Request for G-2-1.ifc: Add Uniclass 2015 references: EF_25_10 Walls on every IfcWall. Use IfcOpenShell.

First a look at what the model holds.

```python
import ifcopenshell

model = ifcopenshell.open("G-2-1.ifc")
print(model.schema)
print("classifications:", [c.Name for c in model.by_type("IfcClassification")])
for ifc_class in ("IfcDoor", "IfcRoof", "IfcStair", "IfcWall", "IfcWindow"):
    print(ifc_class, len(model.by_type(ifc_class)))
```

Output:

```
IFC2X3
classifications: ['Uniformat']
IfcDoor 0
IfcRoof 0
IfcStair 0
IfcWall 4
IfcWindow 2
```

```python
import ifcopenshell
import ifcopenshell.api.classification

model = ifcopenshell.open("G-2-1.ifc")

# IFC2X3 requires Source and Edition and has no link from the project to the system.
system = model.create_entity("IfcClassification", Source="NBS", Edition="2015", Name="Uniclass 2015")

codes = {
    "IfcWall": ("EF_25_10", "Walls"),
}
for ifc_class, (code, name) in codes.items():
    products = model.by_type(ifc_class)
    ifcopenshell.api.classification.add_reference(
        model, products=products, classification=system, identification=code, name=name
    )
    print(code, len(products))

model.write("G-2-1-out.ifc")
```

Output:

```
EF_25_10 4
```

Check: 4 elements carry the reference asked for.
